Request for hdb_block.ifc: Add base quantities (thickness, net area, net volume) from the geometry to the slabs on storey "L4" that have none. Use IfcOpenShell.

First a look at what the model holds.

```python
import ifcopenshell
import ifcopenshell.util.element
import ifcopenshell.util.unit

model = ifcopenshell.open("hdb_block.ifc")
print(model.schema)
for unit_type in ("LENGTHUNIT", "AREAUNIT", "VOLUMEUNIT"):
    print(unit_type, ifcopenshell.util.unit.calculate_unit_scale(model, unit_type))
storey = next(s for s in model.by_type("IfcBuildingStorey") if s.Name == "L4")
slabs = [e for e in ifcopenshell.util.element.get_decomposition(storey) if e.is_a("IfcSlab")]
for e in sorted(slabs, key=lambda e: e.id()):
    print(e.id(), e.is_a(), e.Name, list(ifcopenshell.util.element.get_psets(e, qtos_only=True)), sep=" | ")
```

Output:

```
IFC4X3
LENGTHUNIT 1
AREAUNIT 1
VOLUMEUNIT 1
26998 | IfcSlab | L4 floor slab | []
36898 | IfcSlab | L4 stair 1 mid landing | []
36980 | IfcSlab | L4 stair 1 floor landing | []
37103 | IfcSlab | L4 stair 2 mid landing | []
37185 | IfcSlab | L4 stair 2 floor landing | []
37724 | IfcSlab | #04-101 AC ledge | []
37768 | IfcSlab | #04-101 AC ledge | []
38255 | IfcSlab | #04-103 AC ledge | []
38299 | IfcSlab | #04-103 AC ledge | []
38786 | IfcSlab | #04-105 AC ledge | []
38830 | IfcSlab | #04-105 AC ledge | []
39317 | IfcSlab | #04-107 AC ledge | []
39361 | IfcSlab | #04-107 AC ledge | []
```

```python
import ifcopenshell
import ifcopenshell.api.pset
import ifcopenshell.geom
import ifcopenshell.util.element
import ifcopenshell.util.shape
import ifcopenshell.util.unit

model = ifcopenshell.open("hdb_block.ifc")
unit_scale = ifcopenshell.util.unit.calculate_unit_scale(model)
area_scale = ifcopenshell.util.unit.calculate_unit_scale(model, "AREAUNIT")
volume_scale = ifcopenshell.util.unit.calculate_unit_scale(model, "VOLUMEUNIT")
settings = ifcopenshell.geom.settings()

storey = next(s for s in model.by_type("IfcBuildingStorey") if s.Name == "L4")
slabs = [e for e in ifcopenshell.util.element.get_decomposition(storey) if e.is_a("IfcSlab")]

for e in sorted(slabs, key=lambda e: e.id()):
    if ifcopenshell.util.element.get_psets(e, qtos_only=True, should_inherit=False):
        continue
    # Geometry comes back in metres, in the element's own axes.
    shape = ifcopenshell.geom.create_shape(settings, e)
    values = {
        "Width": ifcopenshell.util.shape.get_z(shape.geometry) / unit_scale,
        "NetArea": ifcopenshell.util.shape.get_footprint_area(shape.geometry) / area_scale,
        "NetVolume": ifcopenshell.util.shape.get_volume(shape.geometry) / volume_scale,
    }
    qto = ifcopenshell.api.pset.add_qto(model, product=e, name="Qto_SlabBaseQuantities")
    ifcopenshell.api.pset.edit_qto(model, qto=qto, properties=values)
    print(e.id(), {k: round(v, 3) for k, v in values.items()})

model.write("hdb_block_v2.ifc")
```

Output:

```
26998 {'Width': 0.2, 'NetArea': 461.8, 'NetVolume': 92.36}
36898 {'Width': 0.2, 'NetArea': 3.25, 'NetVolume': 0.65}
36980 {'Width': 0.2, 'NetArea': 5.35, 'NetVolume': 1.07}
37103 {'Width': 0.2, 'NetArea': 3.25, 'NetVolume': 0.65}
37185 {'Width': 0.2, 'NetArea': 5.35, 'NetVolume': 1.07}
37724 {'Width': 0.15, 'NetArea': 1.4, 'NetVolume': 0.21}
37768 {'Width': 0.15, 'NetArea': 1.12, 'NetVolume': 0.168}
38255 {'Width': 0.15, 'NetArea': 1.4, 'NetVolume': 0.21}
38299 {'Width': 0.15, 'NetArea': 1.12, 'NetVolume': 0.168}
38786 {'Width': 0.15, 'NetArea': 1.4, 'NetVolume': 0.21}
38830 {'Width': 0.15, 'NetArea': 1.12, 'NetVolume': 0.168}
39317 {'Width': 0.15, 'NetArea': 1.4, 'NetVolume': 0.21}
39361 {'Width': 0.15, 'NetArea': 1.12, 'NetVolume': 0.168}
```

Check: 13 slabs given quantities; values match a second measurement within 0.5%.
